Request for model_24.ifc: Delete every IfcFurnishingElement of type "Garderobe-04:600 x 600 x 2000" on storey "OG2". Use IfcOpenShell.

First a look at what the model holds.

```python
import ifcopenshell
import ifcopenshell.util.element

model = ifcopenshell.open("model_24.ifc")
print(model.schema)
storey = next(s for s in model.by_type("IfcBuildingStorey") if s.Name == "OG2")
furniture = [e for e in ifcopenshell.util.element.get_decomposition(storey) if e.is_a("IfcFurnishingElement")]
seen = {}
for e in furniture:
    element_type = ifcopenshell.util.element.get_type(e)
    name = element_type.Name if element_type not in (None, e) else None
    seen[name] = seen.get(name, 0) + 1
for name, count in sorted(seen.items(), key=str):
    print(count, "x", name)
```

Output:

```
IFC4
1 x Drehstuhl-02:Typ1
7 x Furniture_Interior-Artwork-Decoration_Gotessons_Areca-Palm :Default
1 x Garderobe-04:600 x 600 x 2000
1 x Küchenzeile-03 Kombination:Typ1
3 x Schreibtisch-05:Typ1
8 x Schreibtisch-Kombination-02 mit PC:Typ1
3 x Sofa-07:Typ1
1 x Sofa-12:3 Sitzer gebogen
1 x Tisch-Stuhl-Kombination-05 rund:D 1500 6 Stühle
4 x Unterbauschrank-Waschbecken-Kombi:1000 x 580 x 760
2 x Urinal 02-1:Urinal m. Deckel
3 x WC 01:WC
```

```python
import ifcopenshell
import ifcopenshell.api.root
import ifcopenshell.util.element

model = ifcopenshell.open("model_24.ifc")

storey = next(s for s in model.by_type("IfcBuildingStorey") if s.Name == "OG2")
furniture = [e for e in ifcopenshell.util.element.get_decomposition(storey) if e.is_a("IfcFurnishingElement")]
targets = [e for e in furniture if (t := ifcopenshell.util.element.get_type(e)) not in (None, e) and t.Name == "Garderobe-04:600 x 600 x 2000"]

for e in targets:
    ifcopenshell.api.root.remove_product(model, product=e)
print(len(targets), "removed")

model.write("model_24_v2.ifc")
```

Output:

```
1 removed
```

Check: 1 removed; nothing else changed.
